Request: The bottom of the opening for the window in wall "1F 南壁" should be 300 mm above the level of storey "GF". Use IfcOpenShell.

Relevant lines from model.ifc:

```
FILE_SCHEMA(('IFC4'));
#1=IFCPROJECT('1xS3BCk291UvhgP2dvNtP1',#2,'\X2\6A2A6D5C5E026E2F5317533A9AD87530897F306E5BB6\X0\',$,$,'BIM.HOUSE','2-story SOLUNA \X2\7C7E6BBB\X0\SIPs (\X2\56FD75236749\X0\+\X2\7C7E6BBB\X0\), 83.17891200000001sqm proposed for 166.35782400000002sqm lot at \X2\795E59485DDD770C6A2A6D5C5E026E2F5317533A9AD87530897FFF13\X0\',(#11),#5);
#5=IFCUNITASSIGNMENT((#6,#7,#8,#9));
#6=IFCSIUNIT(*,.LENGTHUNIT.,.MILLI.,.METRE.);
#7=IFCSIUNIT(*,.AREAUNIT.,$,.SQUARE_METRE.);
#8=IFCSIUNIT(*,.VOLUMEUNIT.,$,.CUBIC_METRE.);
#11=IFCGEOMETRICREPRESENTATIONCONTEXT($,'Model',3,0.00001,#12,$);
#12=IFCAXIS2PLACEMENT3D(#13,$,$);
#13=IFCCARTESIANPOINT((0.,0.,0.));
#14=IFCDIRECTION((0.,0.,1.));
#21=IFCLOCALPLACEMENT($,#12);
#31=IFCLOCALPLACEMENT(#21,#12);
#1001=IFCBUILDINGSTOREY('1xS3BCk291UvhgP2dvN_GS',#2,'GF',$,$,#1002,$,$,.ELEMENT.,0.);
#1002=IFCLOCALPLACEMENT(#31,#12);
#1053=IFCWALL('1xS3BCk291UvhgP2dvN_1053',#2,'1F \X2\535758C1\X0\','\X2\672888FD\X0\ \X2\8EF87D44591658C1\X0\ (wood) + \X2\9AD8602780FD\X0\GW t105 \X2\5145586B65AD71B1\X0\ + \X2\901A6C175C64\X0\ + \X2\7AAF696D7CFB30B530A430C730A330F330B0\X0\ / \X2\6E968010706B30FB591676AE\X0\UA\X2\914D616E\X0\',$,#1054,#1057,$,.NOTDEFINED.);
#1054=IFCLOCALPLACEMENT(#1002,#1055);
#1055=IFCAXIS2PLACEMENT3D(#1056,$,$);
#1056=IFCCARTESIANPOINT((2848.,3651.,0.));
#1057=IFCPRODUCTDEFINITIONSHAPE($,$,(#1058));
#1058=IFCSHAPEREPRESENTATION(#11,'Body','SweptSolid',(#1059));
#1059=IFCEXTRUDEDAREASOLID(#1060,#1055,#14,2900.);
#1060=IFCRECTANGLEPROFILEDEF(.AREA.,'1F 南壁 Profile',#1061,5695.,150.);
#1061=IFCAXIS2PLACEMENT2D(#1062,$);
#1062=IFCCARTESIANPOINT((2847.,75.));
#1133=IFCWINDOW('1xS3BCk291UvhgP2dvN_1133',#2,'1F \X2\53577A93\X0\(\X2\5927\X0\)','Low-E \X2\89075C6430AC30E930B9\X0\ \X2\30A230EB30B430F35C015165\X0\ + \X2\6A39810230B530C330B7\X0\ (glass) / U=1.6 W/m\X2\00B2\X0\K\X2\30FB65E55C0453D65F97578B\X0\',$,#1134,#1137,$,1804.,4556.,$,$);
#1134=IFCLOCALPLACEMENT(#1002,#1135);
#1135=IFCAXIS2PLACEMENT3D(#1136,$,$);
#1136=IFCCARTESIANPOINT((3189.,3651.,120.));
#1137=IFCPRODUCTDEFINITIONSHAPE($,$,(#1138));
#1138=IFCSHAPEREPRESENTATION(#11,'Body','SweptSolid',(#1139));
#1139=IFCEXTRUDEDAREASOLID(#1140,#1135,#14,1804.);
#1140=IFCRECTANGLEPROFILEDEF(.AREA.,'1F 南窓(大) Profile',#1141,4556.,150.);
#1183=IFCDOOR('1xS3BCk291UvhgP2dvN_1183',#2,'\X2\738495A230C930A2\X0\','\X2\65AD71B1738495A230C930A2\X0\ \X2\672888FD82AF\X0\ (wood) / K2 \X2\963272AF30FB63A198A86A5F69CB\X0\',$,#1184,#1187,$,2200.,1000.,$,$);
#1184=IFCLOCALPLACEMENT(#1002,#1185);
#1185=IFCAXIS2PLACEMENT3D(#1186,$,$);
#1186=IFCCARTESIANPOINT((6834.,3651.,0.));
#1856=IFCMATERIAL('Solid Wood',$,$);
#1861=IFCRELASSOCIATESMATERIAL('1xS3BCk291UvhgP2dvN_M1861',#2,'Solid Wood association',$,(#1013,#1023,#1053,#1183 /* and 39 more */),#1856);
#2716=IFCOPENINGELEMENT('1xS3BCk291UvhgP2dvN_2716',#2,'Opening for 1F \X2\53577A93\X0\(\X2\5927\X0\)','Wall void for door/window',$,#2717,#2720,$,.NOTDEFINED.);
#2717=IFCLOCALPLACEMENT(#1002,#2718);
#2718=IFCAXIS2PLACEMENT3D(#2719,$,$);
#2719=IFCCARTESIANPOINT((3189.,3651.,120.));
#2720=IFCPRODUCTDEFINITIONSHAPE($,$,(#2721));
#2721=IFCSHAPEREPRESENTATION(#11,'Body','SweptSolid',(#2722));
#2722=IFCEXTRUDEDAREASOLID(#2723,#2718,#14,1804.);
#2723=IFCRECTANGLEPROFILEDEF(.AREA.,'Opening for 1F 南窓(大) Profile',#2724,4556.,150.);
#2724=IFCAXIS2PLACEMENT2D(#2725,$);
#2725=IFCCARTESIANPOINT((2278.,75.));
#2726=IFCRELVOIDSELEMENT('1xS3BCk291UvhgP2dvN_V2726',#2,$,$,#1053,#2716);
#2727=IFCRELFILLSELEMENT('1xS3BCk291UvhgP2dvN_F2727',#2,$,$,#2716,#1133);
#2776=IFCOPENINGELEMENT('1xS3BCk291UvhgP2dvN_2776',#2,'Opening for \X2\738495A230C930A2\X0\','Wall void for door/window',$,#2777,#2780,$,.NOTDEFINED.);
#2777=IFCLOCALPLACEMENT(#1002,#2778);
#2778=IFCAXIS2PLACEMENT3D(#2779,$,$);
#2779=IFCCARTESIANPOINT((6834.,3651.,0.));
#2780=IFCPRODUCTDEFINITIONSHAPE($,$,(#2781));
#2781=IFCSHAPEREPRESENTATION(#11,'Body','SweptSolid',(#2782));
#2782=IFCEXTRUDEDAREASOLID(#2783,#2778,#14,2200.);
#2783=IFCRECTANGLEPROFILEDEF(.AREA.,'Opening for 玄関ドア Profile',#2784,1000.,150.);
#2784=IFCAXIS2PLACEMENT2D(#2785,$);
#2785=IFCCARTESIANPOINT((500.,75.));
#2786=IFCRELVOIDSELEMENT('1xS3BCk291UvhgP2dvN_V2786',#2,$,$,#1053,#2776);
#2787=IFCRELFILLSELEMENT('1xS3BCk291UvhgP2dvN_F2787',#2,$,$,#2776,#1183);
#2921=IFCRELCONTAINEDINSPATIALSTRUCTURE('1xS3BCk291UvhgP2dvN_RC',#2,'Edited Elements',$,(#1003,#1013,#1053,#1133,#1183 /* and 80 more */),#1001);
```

```python
import numpy as np
import ifcopenshell
import ifcopenshell.api.geometry
import ifcopenshell.geom
import ifcopenshell.util.element
import ifcopenshell.util.placement
import ifcopenshell.util.shape
import ifcopenshell.util.unit

model = ifcopenshell.open("model.ifc")
unit_scale = ifcopenshell.util.unit.calculate_unit_scale(model)

window = model.by_guid("1xS3BCk291UvhgP2dvN_1133")
opening = window.FillsVoids[0].RelatingOpeningElement
storey = ifcopenshell.util.element.get_container(window, ifc_class="IfcBuildingStorey")
level = ifcopenshell.util.placement.get_local_placement(storey.ObjectPlacement)[2, 3]

# The opening's origin need not be at the sill, so measure its lowest point.
shape = ifcopenshell.geom.create_shape(ifcopenshell.geom.settings(), opening)
bottom = ifcopenshell.util.shape.get_shape_bottom_elevation(shape, shape.geometry) / unit_scale
dz = level + 300.0 - bottom

shift = np.array([0.0, 0.0, dz])
# The window is not placed relative to its opening, so move both.
for product in (opening, window):
    matrix = ifcopenshell.util.placement.get_local_placement(product.ObjectPlacement)
    matrix[:3, 3] += shift
    ifcopenshell.api.geometry.edit_object_placement(model, product=product, matrix=matrix, is_si=False)

print(f"moved by {dz * unit_scale:+.3f} m")

model.write("model_edited.ifc")
```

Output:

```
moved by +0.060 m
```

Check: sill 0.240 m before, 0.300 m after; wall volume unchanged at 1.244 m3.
